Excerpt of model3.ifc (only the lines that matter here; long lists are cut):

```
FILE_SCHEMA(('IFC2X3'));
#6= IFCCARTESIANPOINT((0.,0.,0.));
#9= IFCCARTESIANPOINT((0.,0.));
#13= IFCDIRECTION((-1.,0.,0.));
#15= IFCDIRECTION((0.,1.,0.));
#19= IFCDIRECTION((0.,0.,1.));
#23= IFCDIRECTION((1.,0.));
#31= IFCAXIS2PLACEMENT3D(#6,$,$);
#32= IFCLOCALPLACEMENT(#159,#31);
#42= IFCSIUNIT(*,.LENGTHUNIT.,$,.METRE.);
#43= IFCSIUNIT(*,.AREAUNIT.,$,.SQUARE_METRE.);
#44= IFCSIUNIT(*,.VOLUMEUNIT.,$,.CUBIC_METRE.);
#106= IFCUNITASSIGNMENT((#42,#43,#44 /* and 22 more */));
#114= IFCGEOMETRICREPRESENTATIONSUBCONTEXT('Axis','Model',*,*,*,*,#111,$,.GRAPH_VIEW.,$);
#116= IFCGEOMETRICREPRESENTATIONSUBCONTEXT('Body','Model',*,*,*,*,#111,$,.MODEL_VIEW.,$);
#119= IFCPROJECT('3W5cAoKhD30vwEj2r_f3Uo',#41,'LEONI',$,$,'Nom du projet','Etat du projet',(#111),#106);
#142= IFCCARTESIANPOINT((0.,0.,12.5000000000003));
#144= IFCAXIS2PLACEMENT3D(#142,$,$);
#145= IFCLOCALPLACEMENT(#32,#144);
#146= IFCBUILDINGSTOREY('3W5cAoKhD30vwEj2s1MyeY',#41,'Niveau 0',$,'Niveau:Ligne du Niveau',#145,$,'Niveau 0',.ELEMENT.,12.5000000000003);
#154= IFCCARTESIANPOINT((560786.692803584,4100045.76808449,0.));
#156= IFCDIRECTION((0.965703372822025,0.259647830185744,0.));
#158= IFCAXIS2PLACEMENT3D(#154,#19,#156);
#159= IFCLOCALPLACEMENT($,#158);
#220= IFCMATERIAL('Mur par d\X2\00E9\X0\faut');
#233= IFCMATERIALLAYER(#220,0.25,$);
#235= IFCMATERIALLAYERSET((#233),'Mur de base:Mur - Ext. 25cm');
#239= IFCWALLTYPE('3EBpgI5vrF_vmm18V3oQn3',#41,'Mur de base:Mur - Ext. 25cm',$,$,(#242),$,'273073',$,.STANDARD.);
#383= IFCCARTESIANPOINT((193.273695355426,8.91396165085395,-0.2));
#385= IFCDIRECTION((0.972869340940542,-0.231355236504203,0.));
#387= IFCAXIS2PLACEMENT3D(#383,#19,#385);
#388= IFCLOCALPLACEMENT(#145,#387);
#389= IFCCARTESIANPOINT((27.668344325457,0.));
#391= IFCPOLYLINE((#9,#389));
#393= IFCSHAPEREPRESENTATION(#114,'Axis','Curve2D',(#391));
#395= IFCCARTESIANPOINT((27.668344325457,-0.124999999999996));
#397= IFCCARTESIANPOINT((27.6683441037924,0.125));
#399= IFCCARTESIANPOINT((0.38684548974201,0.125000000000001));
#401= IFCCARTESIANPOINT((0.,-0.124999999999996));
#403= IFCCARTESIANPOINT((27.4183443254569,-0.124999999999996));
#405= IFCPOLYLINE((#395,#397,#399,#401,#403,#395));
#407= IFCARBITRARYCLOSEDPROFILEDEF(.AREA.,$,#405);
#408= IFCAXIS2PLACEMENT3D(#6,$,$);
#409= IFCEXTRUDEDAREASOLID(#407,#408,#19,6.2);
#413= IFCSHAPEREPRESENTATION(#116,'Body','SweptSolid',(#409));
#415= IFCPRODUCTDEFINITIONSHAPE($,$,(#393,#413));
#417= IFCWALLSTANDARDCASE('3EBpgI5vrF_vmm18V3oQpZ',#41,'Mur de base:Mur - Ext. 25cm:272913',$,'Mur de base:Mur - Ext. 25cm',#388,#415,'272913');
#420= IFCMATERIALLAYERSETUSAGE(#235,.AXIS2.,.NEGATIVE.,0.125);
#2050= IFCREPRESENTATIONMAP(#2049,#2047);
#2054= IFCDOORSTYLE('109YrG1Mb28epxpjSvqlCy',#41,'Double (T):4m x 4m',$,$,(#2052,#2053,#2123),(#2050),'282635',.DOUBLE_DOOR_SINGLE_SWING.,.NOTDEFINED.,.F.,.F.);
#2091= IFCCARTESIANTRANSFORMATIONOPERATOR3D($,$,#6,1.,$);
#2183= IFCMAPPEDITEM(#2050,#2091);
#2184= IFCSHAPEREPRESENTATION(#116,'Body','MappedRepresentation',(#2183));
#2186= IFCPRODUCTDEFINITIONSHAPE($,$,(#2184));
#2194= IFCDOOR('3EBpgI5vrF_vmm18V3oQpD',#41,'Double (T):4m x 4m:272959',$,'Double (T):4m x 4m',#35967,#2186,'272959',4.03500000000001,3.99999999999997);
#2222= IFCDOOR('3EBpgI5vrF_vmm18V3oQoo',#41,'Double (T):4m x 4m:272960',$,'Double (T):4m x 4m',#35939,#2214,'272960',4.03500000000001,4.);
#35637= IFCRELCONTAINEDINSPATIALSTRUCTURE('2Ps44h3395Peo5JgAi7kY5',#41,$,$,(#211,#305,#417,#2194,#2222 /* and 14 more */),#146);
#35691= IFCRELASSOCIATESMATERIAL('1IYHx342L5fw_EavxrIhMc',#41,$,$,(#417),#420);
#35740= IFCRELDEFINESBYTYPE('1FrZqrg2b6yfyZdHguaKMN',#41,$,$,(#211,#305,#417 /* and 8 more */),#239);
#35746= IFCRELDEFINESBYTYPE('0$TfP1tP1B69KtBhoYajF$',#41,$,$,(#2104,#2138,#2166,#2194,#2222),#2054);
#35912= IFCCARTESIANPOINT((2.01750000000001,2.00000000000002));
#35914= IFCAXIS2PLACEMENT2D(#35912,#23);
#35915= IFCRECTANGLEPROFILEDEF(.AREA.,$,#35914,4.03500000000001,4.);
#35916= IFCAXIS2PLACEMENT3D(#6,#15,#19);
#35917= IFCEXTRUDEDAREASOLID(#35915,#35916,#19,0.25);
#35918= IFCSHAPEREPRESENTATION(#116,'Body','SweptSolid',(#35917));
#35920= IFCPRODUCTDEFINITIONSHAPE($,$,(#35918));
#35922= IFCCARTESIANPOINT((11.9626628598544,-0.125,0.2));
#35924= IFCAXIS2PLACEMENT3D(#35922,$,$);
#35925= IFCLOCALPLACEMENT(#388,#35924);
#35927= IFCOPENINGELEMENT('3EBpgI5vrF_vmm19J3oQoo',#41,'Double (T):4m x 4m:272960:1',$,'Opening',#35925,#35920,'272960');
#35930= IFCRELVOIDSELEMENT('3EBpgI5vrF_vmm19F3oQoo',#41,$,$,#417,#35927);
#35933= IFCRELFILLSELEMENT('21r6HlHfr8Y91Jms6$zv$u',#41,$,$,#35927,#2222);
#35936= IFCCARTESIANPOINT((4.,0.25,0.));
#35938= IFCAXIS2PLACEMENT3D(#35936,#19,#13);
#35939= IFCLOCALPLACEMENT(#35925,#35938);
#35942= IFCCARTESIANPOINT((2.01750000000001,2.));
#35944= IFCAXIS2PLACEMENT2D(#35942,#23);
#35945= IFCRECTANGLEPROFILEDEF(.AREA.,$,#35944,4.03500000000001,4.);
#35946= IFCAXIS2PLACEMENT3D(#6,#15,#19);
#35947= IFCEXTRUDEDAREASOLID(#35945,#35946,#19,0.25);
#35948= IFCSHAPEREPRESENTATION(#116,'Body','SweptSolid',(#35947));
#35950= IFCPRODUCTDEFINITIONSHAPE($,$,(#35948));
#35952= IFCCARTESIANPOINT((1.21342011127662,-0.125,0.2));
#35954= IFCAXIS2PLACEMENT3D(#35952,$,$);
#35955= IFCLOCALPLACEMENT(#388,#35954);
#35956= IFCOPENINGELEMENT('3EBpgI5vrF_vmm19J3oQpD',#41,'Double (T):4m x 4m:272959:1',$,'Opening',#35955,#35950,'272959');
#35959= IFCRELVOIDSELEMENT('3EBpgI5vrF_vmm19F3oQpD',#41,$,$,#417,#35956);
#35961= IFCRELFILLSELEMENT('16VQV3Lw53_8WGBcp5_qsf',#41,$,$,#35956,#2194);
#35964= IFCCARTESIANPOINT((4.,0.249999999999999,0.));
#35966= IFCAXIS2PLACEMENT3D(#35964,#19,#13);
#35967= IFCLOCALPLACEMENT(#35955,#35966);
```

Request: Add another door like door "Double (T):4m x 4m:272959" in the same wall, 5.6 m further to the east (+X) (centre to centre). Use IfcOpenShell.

```python
import ifcopenshell
import ifcopenshell.api.feature
import ifcopenshell.api.geometry
import ifcopenshell.api.root
import ifcopenshell.geom
import ifcopenshell.util.element
import ifcopenshell.util.placement
import ifcopenshell.util.shape
import ifcopenshell.util.unit

model = ifcopenshell.open("model3.ifc")
unit_scale = ifcopenshell.util.unit.calculate_unit_scale(model)
settings = ifcopenshell.geom.settings()


def volume(element):
    """Net volume in cubic metres, openings subtracted."""
    shape = ifcopenshell.geom.create_shape(settings, element)
    return ifcopenshell.util.shape.get_volume(shape.geometry)


def reuse_history(source, copy):
    """copy_class also copies each property set's owner history, people and application; keep the originals."""
    for rel in copy.IsDefinedBy:
        if rel.is_a("IfcRelDefinesByProperties") and (history := rel.RelatingPropertyDefinition.OwnerHistory):
            rel.RelatingPropertyDefinition.OwnerHistory = source.OwnerHistory
            ifcopenshell.util.element.remove_deep2(model, history)


door = model.by_guid("3EBpgI5vrF_vmm18V3oQpD")
opening = door.FillsVoids[0].RelatingOpeningElement
wall = opening.VoidsElements[0].RelatingBuildingElement
before = volume(wall)
shift = ifcopenshell.util.placement.get_local_placement(wall.ObjectPlacement)[:3, 0] * 5.6 / unit_scale

# copy_class copies the void relationship, type, container and properties, but no geometry.
new_opening = ifcopenshell.api.root.copy_class(model, product=opening)
new_opening.Representation = ifcopenshell.util.element.copy_deep(
    model, opening.Representation, exclude=["IfcGeometricRepresentationContext", "IfcRepresentationMap"]
)
new_opening.Name = "Double (T):4m x 4m"
new_opening.Tag = None
new_door = ifcopenshell.api.root.copy_class(model, product=door)
new_door.Representation = ifcopenshell.util.element.copy_deep(
    model, door.Representation, exclude=["IfcGeometricRepresentationContext", "IfcRepresentationMap"]
)
new_door.Name = "Double (T):4m x 4m"
new_door.Tag = None
reuse_history(door, new_door)
fills = ifcopenshell.api.feature.add_filling(model, opening=new_opening, element=new_door)
fills.OwnerHistory = new_door.OwnerHistory  # required in IFC2X3

for old, new in ((opening, new_opening), (door, new_door)):
    matrix = ifcopenshell.util.placement.get_local_placement(old.ObjectPlacement)
    matrix[:3, 3] += shift
    ifcopenshell.api.geometry.edit_object_placement(model, product=new, matrix=matrix, is_si=False)

after = volume(wall)

print(f"wall volume {before:.3f} -> {after:.3f} m3")

model.write("model3_updated.ifc")
```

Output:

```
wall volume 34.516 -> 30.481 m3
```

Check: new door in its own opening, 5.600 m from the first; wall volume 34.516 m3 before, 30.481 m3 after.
